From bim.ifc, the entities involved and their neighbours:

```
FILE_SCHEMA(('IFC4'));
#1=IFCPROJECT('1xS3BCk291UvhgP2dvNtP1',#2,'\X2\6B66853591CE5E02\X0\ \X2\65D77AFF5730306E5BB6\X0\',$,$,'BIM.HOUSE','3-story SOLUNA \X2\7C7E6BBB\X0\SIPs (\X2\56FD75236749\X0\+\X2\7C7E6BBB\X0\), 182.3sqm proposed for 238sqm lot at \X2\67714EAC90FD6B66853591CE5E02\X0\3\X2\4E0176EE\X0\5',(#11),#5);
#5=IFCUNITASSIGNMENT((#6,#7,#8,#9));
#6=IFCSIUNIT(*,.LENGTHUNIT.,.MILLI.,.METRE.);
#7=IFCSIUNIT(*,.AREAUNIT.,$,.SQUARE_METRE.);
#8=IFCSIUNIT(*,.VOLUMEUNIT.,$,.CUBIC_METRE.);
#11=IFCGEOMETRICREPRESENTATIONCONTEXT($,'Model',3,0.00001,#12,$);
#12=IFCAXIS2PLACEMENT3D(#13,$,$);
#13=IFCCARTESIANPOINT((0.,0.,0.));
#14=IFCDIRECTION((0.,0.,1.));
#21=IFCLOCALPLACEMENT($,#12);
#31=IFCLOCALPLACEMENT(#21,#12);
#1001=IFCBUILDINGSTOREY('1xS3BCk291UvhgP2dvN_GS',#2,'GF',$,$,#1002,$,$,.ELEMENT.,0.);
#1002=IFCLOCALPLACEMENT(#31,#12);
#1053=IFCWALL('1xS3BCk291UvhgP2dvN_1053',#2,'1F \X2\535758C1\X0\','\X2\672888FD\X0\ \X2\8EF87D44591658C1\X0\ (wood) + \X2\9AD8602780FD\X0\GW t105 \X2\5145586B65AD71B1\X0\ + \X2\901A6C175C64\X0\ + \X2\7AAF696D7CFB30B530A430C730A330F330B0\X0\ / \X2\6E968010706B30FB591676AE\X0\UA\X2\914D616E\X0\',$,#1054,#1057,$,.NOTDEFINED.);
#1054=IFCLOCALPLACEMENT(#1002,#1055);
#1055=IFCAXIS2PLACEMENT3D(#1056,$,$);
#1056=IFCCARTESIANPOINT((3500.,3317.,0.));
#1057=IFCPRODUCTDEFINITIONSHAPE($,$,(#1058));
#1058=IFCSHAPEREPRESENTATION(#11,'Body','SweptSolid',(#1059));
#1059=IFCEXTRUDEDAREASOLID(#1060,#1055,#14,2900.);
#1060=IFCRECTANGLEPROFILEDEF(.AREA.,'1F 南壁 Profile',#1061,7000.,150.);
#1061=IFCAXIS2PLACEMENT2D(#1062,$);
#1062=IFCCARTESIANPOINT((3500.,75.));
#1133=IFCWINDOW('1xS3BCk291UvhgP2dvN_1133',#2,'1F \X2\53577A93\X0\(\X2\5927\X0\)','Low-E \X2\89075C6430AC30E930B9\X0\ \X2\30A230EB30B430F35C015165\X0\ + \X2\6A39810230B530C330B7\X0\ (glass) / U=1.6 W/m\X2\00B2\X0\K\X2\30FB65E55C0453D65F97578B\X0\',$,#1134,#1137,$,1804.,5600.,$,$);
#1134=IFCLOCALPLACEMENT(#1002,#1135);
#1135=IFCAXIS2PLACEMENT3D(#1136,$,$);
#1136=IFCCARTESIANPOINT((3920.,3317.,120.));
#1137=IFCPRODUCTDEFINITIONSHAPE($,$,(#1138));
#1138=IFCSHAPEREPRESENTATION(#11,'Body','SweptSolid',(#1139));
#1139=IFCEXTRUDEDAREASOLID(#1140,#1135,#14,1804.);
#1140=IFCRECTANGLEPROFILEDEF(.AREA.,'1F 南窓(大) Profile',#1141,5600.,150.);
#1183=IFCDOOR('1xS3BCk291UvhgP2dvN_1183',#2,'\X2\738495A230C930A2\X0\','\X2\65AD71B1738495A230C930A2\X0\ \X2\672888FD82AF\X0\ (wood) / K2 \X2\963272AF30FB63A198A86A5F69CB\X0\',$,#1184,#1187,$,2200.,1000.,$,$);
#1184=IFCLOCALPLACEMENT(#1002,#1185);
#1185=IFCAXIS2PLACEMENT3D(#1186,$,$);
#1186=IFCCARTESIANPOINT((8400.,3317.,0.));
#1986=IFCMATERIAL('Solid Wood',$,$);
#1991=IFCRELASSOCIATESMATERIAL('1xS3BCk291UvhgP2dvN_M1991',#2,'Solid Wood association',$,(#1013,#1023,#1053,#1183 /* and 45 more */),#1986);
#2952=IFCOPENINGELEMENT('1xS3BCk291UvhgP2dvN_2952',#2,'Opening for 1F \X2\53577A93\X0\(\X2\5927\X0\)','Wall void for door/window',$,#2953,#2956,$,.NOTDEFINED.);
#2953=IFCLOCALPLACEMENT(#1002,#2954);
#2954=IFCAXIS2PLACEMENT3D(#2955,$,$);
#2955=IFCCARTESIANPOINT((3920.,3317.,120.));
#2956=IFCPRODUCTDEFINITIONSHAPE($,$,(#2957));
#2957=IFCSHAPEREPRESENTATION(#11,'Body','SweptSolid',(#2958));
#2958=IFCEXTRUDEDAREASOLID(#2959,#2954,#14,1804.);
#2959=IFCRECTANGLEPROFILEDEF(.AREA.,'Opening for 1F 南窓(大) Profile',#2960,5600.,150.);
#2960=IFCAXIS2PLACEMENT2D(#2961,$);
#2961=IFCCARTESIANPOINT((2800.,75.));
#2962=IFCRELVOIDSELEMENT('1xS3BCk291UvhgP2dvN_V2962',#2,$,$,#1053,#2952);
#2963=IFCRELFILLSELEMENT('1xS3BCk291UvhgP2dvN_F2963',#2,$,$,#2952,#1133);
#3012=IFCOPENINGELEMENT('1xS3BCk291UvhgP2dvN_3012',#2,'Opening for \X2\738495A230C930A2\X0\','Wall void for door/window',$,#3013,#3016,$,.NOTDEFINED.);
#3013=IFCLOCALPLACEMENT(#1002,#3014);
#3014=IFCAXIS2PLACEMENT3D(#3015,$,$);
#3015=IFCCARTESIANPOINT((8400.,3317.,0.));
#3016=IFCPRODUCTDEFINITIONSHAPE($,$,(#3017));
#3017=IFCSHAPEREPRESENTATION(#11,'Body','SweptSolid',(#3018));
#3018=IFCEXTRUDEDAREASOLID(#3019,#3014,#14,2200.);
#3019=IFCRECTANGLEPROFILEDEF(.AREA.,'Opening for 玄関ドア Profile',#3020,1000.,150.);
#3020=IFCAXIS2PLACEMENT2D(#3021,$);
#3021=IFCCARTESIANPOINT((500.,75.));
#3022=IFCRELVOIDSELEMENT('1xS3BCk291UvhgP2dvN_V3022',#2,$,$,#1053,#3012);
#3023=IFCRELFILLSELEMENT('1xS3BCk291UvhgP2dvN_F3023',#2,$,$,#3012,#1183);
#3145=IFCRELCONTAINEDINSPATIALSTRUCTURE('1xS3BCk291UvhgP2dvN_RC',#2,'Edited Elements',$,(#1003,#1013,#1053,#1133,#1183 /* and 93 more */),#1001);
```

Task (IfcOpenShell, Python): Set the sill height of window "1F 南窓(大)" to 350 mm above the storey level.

```python
import numpy as np
import ifcopenshell
import ifcopenshell.api.geometry
import ifcopenshell.geom
import ifcopenshell.util.element
import ifcopenshell.util.placement
import ifcopenshell.util.shape
import ifcopenshell.util.unit

model = ifcopenshell.open("bim.ifc")
unit_scale = ifcopenshell.util.unit.calculate_unit_scale(model)

window = model.by_guid("1xS3BCk291UvhgP2dvN_1133")
opening = window.FillsVoids[0].RelatingOpeningElement
storey = ifcopenshell.util.element.get_container(window, ifc_class="IfcBuildingStorey")
level = ifcopenshell.util.placement.get_local_placement(storey.ObjectPlacement)[2, 3]

# The opening's origin need not be at the sill, so measure its lowest point.
shape = ifcopenshell.geom.create_shape(ifcopenshell.geom.settings(), opening)
bottom = ifcopenshell.util.shape.get_shape_bottom_elevation(shape, shape.geometry) / unit_scale
dz = level + 0.35 / unit_scale - bottom

shift = np.array([0.0, 0.0, dz])
# The window is not placed relative to its opening, so move both.
for product in (opening, window):
    matrix = ifcopenshell.util.placement.get_local_placement(product.ObjectPlacement)
    matrix[:3, 3] += shift
    ifcopenshell.api.geometry.edit_object_placement(model, product=product, matrix=matrix, is_si=False)

print(f"moved by {dz * unit_scale:+.3f} m")

model.write("bim-out.ifc")
```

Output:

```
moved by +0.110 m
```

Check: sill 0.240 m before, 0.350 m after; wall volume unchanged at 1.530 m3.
